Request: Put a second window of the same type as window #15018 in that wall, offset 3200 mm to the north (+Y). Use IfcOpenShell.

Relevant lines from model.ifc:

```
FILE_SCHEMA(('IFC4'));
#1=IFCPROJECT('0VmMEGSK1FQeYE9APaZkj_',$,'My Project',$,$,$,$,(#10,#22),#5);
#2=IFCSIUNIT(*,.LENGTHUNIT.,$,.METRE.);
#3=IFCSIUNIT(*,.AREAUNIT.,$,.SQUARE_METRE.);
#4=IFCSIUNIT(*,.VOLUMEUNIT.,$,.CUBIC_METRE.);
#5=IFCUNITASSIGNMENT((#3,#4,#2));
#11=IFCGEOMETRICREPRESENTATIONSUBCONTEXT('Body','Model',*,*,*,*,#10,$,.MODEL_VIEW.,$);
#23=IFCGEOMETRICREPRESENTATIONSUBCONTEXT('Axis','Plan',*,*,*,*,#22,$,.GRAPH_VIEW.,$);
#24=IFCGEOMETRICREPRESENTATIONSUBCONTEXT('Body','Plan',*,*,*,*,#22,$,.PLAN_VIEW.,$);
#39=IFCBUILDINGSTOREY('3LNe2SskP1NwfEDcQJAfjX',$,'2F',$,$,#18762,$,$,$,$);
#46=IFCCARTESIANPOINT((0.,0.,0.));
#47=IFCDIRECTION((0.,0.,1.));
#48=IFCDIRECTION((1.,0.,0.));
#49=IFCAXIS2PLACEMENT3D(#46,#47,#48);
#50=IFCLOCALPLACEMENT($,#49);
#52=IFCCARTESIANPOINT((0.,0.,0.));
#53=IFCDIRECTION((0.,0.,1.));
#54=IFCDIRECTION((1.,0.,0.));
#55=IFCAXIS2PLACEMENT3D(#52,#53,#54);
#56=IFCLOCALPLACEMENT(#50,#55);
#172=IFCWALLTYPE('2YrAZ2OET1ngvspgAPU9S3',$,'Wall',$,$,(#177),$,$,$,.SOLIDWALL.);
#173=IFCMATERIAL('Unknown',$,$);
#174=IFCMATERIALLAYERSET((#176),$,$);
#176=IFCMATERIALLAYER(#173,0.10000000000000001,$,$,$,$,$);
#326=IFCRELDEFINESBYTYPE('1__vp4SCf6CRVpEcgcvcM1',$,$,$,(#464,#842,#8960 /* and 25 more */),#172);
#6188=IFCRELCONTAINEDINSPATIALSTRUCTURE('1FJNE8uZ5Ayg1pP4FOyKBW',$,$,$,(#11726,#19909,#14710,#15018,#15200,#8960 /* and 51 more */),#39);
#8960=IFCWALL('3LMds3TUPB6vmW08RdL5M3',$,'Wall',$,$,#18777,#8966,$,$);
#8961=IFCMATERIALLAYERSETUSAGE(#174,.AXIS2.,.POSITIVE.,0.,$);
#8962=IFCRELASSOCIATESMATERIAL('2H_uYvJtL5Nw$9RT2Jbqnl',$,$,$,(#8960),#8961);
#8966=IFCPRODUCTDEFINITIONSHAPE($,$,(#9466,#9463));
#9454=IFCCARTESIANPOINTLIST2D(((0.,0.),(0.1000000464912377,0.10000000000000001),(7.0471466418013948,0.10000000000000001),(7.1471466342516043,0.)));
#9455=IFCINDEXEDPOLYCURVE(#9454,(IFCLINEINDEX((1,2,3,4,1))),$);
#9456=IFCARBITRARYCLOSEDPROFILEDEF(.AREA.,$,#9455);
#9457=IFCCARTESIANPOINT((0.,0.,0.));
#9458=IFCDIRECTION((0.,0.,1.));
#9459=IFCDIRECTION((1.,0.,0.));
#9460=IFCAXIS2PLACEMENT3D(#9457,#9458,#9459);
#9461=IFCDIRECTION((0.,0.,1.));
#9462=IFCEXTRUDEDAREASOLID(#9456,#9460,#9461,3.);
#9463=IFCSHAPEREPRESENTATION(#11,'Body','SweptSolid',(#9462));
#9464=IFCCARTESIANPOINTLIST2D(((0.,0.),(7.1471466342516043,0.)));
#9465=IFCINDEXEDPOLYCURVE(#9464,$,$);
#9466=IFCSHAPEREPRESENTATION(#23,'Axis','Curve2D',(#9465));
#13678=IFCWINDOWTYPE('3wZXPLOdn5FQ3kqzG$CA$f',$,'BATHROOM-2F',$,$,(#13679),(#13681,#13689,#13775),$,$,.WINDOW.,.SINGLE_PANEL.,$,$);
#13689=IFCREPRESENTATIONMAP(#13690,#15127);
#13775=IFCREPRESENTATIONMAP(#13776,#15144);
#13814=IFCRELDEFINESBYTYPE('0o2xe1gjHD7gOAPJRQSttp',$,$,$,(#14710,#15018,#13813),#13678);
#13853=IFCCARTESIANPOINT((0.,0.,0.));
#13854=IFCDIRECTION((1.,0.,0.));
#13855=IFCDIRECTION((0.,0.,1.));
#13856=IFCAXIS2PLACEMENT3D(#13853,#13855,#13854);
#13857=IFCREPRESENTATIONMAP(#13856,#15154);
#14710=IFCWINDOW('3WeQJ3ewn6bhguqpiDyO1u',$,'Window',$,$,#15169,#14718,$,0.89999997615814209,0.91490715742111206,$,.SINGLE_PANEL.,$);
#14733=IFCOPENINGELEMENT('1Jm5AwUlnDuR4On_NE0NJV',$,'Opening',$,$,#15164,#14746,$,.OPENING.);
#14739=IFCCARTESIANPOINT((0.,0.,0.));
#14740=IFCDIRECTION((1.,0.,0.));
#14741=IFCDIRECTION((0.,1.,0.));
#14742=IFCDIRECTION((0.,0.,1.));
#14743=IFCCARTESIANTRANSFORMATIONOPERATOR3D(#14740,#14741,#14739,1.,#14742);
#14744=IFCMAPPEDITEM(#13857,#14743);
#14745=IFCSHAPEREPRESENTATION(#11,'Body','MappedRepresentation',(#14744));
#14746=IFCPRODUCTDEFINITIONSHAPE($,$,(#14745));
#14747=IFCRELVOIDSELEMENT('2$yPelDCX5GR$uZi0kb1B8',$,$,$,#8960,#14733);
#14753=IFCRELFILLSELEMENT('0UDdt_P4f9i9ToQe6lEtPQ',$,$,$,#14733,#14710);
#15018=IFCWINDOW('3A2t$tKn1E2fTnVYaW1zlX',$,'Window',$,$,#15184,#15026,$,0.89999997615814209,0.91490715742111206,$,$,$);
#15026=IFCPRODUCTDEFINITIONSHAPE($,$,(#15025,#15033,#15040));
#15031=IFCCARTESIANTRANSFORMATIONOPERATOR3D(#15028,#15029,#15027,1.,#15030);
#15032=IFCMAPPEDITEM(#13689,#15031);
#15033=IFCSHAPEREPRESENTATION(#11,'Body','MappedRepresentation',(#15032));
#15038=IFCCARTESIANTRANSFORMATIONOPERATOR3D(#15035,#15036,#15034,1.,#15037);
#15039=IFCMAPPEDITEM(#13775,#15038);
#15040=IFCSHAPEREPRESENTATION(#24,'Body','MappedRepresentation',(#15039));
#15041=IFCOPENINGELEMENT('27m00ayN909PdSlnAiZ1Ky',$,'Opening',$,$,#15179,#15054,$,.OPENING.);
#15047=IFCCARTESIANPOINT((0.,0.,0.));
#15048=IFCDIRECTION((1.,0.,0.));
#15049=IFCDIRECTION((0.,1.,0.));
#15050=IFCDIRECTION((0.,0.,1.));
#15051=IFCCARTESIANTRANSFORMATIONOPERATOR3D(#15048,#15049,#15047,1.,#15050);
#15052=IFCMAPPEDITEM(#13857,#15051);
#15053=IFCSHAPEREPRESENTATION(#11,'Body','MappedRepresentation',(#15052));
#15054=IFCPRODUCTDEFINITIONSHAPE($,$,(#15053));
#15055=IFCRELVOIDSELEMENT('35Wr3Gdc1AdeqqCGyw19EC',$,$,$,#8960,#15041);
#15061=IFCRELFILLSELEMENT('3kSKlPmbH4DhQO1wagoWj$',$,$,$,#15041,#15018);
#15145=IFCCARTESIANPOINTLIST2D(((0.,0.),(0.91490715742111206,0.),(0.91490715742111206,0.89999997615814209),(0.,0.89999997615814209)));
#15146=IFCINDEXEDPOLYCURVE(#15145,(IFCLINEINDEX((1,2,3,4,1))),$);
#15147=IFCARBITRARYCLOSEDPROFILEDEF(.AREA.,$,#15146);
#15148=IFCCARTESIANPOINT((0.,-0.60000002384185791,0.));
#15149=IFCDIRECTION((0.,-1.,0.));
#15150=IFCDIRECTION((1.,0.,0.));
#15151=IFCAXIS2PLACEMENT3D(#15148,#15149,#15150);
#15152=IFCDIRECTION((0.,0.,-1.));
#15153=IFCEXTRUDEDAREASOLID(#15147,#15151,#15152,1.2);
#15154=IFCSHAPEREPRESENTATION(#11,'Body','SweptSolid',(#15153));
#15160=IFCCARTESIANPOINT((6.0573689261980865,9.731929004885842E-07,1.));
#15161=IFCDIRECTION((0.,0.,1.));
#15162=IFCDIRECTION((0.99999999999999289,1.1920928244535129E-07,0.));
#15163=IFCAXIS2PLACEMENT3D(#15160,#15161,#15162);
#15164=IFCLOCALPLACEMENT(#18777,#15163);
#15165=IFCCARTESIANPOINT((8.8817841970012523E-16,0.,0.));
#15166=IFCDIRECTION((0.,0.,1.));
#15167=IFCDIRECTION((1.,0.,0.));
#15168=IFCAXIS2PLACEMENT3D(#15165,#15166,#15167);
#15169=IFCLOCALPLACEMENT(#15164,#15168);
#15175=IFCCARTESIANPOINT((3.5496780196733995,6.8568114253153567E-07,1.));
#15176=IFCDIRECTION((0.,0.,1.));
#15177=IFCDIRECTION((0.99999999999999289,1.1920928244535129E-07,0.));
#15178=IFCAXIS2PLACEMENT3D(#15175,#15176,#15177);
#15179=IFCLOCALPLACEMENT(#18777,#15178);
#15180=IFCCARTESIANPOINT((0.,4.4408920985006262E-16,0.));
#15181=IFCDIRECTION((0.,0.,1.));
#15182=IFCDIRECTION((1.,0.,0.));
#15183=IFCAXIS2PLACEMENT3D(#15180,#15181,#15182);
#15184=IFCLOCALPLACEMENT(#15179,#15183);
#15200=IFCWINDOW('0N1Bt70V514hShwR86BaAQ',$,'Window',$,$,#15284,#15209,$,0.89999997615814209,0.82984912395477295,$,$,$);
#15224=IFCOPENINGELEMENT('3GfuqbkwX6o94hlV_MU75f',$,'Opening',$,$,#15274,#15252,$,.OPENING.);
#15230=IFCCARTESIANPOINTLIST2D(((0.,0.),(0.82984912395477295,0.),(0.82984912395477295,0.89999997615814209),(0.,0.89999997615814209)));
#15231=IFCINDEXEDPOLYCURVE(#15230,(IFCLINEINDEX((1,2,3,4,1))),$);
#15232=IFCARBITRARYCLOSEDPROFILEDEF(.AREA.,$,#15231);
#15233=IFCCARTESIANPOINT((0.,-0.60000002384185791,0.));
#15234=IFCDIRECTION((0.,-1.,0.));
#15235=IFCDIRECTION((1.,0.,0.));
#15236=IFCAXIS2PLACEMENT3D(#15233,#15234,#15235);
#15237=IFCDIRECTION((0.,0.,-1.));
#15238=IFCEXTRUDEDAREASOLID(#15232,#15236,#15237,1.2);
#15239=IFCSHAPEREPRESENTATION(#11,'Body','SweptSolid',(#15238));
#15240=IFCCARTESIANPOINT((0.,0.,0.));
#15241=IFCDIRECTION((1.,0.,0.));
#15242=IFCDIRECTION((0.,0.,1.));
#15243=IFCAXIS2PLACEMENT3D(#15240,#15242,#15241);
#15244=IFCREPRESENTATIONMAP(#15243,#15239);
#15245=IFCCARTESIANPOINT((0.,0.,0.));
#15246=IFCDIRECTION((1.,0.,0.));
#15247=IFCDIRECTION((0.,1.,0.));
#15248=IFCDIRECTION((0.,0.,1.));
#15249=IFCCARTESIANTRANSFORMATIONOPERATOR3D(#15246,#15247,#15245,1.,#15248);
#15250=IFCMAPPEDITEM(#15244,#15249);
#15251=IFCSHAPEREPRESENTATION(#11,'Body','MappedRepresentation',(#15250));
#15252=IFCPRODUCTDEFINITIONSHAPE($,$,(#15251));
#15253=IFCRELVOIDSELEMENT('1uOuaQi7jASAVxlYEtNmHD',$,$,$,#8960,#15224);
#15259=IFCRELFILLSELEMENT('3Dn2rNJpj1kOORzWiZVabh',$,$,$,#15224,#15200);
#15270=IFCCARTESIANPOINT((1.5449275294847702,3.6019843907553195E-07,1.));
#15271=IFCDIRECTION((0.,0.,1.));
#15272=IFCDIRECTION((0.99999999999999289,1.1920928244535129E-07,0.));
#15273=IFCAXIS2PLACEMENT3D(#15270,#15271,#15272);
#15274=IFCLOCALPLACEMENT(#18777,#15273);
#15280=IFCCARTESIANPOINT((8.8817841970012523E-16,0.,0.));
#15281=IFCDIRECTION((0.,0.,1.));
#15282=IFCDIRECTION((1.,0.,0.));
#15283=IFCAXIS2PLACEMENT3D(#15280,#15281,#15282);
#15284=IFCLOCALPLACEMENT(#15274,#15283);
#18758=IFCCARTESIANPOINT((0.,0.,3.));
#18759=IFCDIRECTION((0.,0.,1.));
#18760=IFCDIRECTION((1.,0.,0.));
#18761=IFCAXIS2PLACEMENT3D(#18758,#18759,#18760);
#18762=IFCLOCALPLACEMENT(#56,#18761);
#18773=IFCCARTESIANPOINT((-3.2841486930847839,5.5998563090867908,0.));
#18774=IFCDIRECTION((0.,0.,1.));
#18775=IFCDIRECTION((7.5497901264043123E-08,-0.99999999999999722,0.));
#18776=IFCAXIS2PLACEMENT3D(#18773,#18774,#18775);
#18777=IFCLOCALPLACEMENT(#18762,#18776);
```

```python
import ifcopenshell
import ifcopenshell.api.feature
import ifcopenshell.api.geometry
import ifcopenshell.api.root
import ifcopenshell.geom
import ifcopenshell.util.element
import ifcopenshell.util.placement
import ifcopenshell.util.shape
import ifcopenshell.util.unit

model = ifcopenshell.open("model.ifc")
unit_scale = ifcopenshell.util.unit.calculate_unit_scale(model)
settings = ifcopenshell.geom.settings()


def volume(element):
    """Net volume in cubic metres, openings subtracted."""
    shape = ifcopenshell.geom.create_shape(settings, element)
    return ifcopenshell.util.shape.get_volume(shape.geometry)


window = model.by_guid("3A2t$tKn1E2fTnVYaW1zlX")
opening = window.FillsVoids[0].RelatingOpeningElement
wall = opening.VoidsElements[0].RelatingBuildingElement
before = volume(wall)
shift = ifcopenshell.util.placement.get_local_placement(wall.ObjectPlacement)[:3, 0] * -3.2 / unit_scale

# copy_class copies the void relationship, type, container and properties, but no geometry.
new_opening = ifcopenshell.api.root.copy_class(model, product=opening)
new_opening.Representation = ifcopenshell.util.element.copy_deep(
    model, opening.Representation, exclude=["IfcGeometricRepresentationContext", "IfcRepresentationMap"]
)
new_window = ifcopenshell.api.root.copy_class(model, product=window)
new_window.Representation = ifcopenshell.util.element.copy_deep(
    model, window.Representation, exclude=["IfcGeometricRepresentationContext", "IfcRepresentationMap"]
)
ifcopenshell.api.feature.add_filling(model, opening=new_opening, element=new_window)

for old, new in ((opening, new_opening), (window, new_window)):
    matrix = ifcopenshell.util.placement.get_local_placement(old.ObjectPlacement)
    matrix[:3, 3] += shift
    ifcopenshell.api.geometry.edit_object_placement(model, product=new, matrix=matrix, is_si=False)

after = volume(wall)

print(f"wall volume {before:.3f} -> {after:.3f} m3")

model.write("model_rev.ifc")
```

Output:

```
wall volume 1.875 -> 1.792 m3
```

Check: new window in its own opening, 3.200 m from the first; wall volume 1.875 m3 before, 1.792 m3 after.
